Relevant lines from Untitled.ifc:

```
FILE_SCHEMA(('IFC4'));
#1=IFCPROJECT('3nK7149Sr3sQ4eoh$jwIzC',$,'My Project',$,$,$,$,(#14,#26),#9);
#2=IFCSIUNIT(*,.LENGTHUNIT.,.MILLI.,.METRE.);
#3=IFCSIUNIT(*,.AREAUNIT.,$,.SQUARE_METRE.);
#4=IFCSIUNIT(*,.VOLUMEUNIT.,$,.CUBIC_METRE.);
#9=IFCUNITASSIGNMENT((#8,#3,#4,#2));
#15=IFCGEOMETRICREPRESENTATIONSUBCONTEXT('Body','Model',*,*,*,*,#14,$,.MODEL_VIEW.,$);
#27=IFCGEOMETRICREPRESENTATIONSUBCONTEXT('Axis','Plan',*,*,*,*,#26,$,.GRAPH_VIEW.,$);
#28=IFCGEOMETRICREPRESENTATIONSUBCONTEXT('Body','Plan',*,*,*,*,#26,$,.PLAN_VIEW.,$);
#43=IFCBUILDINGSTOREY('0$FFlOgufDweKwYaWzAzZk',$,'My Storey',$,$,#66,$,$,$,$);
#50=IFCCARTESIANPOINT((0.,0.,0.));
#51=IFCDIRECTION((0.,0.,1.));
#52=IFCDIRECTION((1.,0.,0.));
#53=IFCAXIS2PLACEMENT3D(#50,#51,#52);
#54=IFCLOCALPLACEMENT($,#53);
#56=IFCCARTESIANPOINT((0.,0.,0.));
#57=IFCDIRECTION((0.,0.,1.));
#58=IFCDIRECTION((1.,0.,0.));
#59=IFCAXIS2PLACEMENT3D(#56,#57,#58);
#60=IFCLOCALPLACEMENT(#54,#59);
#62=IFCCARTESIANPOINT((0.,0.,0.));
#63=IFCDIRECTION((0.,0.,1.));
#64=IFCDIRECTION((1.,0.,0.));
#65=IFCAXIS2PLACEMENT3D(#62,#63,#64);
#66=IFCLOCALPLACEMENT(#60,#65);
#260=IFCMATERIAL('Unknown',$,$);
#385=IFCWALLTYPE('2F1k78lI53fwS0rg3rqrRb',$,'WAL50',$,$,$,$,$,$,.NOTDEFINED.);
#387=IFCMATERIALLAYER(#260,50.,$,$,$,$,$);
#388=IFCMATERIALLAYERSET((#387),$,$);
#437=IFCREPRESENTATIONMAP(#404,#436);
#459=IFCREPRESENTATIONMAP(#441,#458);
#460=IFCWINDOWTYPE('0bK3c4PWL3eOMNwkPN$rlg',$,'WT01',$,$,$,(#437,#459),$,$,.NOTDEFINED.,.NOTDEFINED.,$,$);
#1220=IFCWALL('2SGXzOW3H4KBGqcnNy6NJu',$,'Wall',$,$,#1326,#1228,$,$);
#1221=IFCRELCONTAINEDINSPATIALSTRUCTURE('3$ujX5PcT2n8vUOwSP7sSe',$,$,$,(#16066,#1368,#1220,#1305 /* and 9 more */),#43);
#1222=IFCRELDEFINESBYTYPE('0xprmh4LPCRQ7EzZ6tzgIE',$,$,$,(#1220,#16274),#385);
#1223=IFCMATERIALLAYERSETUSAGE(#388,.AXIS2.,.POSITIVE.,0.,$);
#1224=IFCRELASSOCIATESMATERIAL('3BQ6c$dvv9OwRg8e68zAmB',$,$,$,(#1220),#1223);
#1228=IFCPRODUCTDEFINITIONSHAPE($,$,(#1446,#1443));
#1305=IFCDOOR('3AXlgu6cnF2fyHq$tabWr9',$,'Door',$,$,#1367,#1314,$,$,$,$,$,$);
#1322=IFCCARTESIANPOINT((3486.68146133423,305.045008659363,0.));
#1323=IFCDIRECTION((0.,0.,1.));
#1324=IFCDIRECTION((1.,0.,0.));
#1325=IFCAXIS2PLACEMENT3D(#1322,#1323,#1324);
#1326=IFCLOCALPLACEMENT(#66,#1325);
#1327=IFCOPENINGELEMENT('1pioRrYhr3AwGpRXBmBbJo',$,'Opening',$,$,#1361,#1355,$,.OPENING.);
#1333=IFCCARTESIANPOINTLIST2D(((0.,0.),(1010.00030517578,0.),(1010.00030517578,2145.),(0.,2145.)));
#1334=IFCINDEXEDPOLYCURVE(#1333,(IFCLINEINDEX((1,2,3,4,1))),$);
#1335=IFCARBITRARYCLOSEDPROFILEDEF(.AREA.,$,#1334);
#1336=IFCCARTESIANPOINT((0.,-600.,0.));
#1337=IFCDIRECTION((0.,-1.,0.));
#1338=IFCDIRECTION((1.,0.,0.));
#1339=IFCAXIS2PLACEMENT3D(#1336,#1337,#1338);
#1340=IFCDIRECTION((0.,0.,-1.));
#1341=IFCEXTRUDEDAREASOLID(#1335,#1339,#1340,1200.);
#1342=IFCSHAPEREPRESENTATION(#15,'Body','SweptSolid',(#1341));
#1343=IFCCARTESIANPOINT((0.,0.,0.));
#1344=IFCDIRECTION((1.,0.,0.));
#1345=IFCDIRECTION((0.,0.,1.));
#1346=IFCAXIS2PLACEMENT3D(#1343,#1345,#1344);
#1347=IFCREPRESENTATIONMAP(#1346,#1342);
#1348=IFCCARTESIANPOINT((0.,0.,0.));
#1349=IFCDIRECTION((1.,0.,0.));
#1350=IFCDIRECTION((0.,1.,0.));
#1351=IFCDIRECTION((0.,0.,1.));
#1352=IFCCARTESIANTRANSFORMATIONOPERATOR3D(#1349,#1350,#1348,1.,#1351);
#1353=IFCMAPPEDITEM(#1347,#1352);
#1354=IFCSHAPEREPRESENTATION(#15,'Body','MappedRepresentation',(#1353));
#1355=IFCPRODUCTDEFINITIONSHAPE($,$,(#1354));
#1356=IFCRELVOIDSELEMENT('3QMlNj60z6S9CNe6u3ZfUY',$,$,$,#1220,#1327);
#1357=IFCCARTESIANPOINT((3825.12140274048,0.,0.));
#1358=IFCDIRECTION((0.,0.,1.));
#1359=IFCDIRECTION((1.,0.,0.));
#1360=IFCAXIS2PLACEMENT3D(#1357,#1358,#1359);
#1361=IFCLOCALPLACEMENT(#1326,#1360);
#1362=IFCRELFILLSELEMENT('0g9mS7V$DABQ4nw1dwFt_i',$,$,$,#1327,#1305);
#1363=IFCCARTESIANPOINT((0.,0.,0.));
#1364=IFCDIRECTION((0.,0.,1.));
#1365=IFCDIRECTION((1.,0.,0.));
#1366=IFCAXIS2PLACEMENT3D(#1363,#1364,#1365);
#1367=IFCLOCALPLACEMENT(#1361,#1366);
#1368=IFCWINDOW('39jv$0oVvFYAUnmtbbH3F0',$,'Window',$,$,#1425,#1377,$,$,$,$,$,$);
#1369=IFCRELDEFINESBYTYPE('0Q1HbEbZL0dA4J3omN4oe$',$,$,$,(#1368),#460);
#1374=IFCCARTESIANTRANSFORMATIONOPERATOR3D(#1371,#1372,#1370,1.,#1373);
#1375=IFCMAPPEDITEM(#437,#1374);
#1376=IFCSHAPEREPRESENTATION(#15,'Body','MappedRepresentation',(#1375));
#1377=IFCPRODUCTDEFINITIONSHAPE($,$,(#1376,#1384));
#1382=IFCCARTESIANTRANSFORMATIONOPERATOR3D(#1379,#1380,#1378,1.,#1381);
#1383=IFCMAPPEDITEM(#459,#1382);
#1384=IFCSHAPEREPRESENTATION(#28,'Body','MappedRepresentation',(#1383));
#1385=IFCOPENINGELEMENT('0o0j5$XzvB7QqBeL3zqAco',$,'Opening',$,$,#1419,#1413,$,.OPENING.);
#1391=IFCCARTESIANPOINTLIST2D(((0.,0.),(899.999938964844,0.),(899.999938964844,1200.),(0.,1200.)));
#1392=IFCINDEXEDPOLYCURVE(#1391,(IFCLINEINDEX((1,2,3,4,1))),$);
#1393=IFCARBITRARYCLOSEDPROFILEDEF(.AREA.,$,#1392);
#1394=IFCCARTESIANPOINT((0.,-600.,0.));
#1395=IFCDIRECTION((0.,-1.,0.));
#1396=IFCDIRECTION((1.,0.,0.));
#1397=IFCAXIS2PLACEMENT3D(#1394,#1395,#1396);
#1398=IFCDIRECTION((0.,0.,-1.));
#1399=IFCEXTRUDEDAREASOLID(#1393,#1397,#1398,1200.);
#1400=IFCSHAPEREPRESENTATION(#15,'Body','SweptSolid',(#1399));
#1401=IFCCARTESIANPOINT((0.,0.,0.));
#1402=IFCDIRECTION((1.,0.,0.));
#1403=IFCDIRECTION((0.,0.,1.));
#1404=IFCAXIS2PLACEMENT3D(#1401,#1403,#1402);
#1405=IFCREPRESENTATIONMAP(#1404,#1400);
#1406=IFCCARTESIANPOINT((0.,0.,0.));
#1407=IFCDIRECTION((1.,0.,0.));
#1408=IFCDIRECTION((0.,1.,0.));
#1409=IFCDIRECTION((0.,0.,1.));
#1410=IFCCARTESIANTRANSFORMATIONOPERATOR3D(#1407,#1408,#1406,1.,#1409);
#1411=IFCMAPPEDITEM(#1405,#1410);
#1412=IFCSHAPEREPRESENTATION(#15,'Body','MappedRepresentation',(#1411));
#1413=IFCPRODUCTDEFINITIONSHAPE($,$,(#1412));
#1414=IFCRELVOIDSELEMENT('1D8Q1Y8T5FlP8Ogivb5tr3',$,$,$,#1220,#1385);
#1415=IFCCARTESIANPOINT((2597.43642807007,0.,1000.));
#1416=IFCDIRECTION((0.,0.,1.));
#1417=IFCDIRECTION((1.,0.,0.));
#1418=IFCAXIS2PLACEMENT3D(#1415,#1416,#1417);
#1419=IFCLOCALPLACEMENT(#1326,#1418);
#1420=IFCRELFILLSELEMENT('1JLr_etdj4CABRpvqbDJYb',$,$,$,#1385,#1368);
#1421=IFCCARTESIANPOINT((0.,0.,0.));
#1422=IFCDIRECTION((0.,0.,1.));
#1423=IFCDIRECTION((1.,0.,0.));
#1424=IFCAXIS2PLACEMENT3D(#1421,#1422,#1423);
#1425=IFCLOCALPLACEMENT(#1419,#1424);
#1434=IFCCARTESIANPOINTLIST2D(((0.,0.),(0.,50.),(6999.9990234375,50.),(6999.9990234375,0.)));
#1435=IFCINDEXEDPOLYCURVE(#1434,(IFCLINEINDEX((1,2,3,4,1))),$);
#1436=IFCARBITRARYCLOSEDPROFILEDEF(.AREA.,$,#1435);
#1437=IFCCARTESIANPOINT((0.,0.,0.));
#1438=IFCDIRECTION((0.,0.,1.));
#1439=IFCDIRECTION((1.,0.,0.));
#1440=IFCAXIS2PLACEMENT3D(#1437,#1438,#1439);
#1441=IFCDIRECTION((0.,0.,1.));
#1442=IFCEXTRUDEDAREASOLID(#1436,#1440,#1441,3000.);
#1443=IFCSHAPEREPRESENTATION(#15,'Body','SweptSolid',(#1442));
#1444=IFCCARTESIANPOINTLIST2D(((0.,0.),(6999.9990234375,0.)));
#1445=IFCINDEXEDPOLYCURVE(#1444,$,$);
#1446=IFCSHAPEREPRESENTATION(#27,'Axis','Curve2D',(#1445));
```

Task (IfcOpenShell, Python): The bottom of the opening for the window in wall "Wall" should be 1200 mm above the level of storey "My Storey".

```python
import numpy as np
import ifcopenshell
import ifcopenshell.api.geometry
import ifcopenshell.geom
import ifcopenshell.util.element
import ifcopenshell.util.placement
import ifcopenshell.util.shape
import ifcopenshell.util.unit

model = ifcopenshell.open("Untitled.ifc")
unit_scale = ifcopenshell.util.unit.calculate_unit_scale(model)

window = model.by_guid("39jv$0oVvFYAUnmtbbH3F0")
opening = window.FillsVoids[0].RelatingOpeningElement
storey = ifcopenshell.util.element.get_container(window, ifc_class="IfcBuildingStorey")
level = ifcopenshell.util.placement.get_local_placement(storey.ObjectPlacement)[2, 3]

# The opening's origin need not be at the sill, so measure its lowest point.
shape = ifcopenshell.geom.create_shape(ifcopenshell.geom.settings(), opening)
bottom = ifcopenshell.util.shape.get_shape_bottom_elevation(shape, shape.geometry) / unit_scale
dz = level + 1200.0 - bottom

shift = np.array([0.0, 0.0, dz])
# The window is placed relative to its opening, so it follows when the opening moves.
matrix = ifcopenshell.util.placement.get_local_placement(opening.ObjectPlacement)
matrix[:3, 3] += shift
ifcopenshell.api.geometry.edit_object_placement(
    model, product=opening, matrix=matrix, is_si=False, should_transform_children=True
)

print(f"moved by {dz * unit_scale:+.3f} m")

model.write("Untitled_updated.ifc")
```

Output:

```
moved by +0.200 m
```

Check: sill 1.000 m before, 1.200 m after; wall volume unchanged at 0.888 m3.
